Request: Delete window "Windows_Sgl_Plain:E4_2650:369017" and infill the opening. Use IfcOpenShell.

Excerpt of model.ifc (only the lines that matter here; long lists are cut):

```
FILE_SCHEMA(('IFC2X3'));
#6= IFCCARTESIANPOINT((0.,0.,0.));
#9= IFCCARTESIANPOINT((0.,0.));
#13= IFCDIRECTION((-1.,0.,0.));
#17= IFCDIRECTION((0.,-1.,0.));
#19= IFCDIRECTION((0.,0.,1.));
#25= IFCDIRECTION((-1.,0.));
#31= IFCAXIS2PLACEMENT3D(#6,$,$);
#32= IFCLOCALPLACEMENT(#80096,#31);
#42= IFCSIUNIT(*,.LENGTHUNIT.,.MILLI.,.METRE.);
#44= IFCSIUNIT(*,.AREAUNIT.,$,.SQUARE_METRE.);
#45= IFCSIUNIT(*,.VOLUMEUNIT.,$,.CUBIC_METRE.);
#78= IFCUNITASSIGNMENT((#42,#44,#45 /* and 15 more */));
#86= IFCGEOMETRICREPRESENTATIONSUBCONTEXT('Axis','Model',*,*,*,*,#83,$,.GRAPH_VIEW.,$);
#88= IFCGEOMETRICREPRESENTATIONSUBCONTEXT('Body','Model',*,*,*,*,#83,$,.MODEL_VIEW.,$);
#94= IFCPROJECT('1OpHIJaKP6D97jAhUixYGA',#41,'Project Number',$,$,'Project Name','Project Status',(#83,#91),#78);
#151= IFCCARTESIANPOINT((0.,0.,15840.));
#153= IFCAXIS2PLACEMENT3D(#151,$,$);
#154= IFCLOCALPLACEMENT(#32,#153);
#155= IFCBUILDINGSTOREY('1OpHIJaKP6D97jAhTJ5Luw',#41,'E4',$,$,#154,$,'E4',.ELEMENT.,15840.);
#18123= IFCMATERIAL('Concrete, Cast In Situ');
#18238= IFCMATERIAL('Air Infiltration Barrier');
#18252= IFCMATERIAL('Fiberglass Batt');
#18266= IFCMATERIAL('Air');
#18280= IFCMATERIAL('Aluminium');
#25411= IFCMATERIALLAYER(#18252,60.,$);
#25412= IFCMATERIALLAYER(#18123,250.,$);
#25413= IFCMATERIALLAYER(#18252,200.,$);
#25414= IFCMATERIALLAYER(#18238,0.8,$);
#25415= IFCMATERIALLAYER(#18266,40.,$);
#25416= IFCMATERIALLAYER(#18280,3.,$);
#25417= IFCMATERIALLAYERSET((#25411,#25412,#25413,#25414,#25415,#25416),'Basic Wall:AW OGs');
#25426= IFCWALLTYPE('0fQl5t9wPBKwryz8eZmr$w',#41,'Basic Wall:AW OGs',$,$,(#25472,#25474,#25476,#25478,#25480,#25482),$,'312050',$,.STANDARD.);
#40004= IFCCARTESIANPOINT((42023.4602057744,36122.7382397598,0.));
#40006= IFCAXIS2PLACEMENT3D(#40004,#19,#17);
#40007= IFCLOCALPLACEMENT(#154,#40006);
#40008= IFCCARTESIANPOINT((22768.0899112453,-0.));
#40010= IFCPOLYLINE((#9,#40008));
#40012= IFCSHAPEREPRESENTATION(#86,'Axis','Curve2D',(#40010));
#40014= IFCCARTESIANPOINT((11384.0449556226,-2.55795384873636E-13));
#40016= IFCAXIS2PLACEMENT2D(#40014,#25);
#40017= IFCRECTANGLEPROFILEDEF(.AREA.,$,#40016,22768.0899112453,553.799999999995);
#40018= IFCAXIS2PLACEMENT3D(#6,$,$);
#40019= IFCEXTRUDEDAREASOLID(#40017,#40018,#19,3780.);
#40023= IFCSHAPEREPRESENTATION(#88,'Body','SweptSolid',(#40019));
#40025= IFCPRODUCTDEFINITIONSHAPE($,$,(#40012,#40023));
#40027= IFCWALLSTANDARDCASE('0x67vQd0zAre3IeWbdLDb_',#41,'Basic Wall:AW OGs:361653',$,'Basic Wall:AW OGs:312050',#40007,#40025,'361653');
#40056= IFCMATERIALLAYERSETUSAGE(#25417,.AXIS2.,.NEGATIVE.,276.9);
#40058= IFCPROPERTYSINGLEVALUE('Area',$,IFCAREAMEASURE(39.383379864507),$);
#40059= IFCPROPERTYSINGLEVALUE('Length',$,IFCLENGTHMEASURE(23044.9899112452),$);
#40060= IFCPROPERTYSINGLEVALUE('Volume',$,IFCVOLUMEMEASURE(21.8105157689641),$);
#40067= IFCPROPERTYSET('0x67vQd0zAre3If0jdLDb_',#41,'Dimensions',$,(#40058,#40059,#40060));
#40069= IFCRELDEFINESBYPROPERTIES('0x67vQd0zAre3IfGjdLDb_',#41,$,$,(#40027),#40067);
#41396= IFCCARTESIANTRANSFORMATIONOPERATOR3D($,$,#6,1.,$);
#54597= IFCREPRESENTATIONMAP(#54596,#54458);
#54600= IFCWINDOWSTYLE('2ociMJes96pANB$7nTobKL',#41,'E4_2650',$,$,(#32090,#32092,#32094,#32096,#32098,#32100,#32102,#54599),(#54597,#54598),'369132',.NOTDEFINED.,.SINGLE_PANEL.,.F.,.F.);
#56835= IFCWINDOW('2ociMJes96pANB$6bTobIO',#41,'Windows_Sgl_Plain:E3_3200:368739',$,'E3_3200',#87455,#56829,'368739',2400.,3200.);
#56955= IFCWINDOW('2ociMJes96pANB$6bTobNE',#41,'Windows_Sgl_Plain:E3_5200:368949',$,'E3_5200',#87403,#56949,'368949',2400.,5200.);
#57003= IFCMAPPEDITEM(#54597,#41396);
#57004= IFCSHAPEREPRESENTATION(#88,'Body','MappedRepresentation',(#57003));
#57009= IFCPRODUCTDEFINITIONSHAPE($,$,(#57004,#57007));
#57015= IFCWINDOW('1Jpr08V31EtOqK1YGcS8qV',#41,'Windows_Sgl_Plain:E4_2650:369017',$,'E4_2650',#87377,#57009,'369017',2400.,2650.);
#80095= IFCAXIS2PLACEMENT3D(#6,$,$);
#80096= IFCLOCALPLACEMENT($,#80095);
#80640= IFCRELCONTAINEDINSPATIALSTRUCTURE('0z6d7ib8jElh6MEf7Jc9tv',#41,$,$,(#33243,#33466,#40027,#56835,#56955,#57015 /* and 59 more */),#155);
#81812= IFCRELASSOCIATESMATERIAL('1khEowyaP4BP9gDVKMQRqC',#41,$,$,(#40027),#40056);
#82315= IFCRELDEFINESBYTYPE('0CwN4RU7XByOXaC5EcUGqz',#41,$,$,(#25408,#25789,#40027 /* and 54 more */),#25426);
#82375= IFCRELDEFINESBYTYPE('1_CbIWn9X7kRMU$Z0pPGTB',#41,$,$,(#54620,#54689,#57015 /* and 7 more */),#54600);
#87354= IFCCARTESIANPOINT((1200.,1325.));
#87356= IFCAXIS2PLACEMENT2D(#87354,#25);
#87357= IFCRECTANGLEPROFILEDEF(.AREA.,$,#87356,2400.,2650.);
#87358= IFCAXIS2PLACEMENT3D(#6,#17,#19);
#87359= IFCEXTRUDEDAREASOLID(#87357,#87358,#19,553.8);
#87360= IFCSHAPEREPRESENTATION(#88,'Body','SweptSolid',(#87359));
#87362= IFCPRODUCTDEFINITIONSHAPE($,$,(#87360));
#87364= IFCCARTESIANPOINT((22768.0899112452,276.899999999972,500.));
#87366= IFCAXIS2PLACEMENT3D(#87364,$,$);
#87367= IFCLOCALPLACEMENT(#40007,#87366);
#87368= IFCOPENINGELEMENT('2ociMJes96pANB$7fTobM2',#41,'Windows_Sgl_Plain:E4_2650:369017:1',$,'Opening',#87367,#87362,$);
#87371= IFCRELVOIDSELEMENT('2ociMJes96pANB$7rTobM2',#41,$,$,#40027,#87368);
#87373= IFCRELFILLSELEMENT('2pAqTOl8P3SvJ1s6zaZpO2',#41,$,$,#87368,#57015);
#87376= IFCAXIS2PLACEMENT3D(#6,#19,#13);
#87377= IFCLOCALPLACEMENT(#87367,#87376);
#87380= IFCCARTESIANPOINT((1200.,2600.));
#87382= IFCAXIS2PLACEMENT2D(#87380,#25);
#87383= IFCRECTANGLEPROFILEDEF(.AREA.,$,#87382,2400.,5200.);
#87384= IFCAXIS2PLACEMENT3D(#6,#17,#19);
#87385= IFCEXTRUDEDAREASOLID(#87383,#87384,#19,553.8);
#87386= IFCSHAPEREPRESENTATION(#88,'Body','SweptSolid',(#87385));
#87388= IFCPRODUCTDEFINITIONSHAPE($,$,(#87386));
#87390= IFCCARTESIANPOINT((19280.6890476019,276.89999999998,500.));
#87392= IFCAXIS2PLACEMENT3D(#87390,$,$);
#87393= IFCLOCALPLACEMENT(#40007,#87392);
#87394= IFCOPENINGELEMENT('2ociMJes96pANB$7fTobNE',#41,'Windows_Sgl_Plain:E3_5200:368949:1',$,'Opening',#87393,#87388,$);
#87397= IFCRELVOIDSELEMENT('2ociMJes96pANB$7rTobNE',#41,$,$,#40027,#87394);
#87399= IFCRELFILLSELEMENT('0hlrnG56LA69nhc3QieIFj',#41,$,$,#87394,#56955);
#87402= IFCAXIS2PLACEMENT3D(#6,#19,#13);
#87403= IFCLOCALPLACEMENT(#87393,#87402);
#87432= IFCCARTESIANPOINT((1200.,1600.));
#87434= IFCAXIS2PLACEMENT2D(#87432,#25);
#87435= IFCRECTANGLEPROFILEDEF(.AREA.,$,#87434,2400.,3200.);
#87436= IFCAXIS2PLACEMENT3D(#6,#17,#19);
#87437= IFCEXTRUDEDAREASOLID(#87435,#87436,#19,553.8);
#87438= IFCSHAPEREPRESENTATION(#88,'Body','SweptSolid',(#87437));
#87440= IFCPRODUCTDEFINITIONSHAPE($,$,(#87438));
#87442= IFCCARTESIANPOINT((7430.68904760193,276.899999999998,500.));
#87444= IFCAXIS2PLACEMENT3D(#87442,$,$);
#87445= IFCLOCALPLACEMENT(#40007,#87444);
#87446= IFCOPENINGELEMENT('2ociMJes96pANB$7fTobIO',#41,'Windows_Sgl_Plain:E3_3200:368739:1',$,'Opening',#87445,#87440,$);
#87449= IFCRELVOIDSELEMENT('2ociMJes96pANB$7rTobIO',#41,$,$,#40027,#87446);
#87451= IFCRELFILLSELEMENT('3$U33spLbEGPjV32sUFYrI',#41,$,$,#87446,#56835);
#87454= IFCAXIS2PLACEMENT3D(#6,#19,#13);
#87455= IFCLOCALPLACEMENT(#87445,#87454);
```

```python
import ifcopenshell
import ifcopenshell.api.feature
import ifcopenshell.api.pset
import ifcopenshell.api.root
import ifcopenshell.geom
import ifcopenshell.util.element
import ifcopenshell.util.shape
import ifcopenshell.util.unit

model = ifcopenshell.open("model.ifc")
area_scale = ifcopenshell.util.unit.calculate_unit_scale(model, "AREAUNIT")
volume_scale = ifcopenshell.util.unit.calculate_unit_scale(model, "VOLUMEUNIT")
settings = ifcopenshell.geom.settings()


def volume(element):
    """Net volume in cubic metres, openings subtracted."""
    shape = ifcopenshell.geom.create_shape(settings, element)
    return ifcopenshell.util.shape.get_volume(shape.geometry)


window = model.by_guid("1Jpr08V31EtOqK1YGcS8qV")
opening = window.FillsVoids[0].RelatingOpeningElement
wall = opening.VoidsElements[0].RelatingBuildingElement
before = volume(wall)

ifcopenshell.api.root.remove_product(model, product=window)
ifcopenshell.api.feature.remove_feature(model, feature=opening)

after = volume(wall)
thickness = 0.5538  # wall thickness in metres

# Update the wall's stored quantities.
pset = model.by_id(ifcopenshell.util.element.get_pset(wall, "Dimensions", should_inherit=False)["id"])
ifcopenshell.api.pset.edit_pset(model, pset=pset, properties={
    "Area": model.create_entity("IfcAreaMeasure", after / thickness / area_scale),
    "Volume": model.create_entity("IfcVolumeMeasure", after / volume_scale),
})

print(f"wall volume {before:.3f} -> {after:.3f} m3")

model.write("model-out.ifc")
```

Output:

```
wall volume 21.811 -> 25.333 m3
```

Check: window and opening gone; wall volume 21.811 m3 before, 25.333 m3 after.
